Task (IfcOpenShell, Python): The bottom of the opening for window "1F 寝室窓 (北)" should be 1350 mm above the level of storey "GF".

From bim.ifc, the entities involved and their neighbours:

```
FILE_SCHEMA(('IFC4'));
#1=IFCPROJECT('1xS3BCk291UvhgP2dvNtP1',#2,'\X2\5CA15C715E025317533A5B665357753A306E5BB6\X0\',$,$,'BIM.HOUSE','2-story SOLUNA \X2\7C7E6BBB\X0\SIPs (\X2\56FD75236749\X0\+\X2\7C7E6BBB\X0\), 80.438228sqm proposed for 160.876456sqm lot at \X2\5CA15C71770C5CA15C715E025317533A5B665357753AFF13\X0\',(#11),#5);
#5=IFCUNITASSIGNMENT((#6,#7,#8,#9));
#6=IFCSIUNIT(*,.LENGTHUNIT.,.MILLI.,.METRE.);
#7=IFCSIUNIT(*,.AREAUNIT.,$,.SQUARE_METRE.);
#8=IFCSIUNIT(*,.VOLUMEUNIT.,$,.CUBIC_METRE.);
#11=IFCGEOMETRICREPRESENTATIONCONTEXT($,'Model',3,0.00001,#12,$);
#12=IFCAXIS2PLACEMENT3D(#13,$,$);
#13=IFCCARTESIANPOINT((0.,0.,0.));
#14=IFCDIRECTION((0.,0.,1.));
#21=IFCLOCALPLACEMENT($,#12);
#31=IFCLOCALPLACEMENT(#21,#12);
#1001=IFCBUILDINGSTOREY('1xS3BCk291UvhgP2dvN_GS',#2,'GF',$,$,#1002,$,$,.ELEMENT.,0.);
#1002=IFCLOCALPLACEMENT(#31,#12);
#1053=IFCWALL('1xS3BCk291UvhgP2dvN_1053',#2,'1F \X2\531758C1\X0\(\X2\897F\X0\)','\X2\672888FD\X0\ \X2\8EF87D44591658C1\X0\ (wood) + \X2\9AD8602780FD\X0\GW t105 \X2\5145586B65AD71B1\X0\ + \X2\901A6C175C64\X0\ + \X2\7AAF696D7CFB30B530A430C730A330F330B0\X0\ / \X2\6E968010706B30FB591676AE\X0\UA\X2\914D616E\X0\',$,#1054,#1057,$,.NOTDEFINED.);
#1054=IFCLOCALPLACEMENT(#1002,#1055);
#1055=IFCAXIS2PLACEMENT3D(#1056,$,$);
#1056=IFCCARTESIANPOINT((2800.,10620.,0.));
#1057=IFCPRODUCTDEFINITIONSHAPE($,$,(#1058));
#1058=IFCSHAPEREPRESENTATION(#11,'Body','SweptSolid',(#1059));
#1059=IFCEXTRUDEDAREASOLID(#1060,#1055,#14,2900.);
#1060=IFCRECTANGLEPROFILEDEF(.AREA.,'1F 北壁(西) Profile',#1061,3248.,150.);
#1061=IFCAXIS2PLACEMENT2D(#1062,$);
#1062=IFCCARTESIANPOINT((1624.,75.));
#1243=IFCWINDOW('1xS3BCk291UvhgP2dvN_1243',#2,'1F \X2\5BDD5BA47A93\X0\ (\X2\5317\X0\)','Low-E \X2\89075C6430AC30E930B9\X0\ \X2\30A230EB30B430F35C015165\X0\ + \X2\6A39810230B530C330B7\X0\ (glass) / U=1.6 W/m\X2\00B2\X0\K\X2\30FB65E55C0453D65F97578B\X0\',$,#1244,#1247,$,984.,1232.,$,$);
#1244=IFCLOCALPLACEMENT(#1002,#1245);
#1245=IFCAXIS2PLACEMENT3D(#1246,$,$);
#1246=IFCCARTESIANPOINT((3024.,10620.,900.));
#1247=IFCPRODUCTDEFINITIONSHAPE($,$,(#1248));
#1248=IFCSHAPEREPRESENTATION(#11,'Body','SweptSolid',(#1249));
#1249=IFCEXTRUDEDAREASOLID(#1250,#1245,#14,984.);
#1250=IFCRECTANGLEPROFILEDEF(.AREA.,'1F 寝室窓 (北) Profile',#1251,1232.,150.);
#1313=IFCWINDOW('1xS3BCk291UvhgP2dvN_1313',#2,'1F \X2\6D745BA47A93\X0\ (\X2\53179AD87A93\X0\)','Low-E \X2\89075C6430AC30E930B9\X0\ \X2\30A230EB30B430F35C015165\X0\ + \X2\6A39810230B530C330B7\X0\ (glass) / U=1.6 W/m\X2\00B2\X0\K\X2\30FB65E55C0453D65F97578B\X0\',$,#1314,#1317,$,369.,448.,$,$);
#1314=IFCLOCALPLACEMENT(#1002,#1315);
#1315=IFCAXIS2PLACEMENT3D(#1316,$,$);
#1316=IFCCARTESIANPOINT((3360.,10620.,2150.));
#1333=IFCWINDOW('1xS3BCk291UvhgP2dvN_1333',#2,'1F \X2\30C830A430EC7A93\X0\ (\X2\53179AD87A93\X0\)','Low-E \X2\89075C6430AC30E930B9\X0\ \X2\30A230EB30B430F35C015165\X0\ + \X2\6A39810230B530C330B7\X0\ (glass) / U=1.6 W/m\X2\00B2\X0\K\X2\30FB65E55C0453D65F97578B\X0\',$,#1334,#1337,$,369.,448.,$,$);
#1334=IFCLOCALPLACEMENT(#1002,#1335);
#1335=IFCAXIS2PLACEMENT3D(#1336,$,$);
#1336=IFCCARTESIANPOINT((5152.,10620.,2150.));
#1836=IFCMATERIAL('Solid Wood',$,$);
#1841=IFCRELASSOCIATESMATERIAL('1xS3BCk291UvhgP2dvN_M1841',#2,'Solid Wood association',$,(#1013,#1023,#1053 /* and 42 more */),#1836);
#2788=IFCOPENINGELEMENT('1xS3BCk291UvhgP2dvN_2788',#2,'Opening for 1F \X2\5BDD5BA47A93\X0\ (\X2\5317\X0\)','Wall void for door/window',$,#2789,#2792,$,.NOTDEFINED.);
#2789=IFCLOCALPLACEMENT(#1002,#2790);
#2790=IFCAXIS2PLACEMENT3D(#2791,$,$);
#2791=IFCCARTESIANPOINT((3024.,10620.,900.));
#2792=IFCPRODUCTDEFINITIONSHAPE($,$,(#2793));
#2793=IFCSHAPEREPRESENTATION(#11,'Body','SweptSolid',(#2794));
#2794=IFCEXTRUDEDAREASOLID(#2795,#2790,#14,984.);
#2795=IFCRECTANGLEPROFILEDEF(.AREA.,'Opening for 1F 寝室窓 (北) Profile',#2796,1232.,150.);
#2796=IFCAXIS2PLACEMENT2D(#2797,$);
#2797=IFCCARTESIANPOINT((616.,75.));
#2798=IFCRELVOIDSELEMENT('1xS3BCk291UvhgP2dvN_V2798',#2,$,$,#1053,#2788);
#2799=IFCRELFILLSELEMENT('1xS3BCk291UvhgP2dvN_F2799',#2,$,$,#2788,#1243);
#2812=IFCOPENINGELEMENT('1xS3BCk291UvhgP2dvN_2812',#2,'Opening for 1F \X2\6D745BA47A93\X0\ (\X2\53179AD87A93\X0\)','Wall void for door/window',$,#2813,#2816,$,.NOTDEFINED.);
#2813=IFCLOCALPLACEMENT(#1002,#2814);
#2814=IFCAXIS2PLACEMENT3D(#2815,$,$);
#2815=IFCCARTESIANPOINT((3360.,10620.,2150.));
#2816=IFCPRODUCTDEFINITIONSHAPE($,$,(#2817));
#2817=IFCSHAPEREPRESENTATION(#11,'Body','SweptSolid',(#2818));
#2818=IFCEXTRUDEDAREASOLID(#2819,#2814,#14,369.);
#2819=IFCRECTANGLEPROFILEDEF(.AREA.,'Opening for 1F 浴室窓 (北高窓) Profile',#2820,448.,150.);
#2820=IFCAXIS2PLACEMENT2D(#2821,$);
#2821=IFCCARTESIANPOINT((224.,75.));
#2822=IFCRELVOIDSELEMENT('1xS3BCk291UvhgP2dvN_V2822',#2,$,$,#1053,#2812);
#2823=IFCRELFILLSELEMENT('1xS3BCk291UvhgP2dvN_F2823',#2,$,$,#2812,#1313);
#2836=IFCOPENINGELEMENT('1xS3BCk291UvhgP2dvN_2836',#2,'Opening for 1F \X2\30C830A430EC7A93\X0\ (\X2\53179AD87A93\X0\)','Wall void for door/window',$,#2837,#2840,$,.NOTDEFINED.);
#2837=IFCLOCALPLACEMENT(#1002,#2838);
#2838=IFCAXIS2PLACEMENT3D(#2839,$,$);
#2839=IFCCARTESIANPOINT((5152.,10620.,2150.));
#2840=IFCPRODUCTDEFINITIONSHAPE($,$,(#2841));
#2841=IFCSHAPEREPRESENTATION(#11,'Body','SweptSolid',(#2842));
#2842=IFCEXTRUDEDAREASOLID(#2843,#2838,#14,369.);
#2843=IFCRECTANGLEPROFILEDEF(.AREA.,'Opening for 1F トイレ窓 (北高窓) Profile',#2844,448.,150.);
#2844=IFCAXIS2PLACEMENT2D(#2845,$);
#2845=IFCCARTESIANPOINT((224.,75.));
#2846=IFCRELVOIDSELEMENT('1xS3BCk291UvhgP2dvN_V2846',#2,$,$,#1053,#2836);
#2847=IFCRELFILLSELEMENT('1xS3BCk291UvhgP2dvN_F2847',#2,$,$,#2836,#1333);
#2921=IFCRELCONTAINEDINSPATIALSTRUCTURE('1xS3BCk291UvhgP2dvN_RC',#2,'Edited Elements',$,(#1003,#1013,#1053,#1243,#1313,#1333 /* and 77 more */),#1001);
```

```python
import numpy as np
import ifcopenshell
import ifcopenshell.api.geometry
import ifcopenshell.geom
import ifcopenshell.util.element
import ifcopenshell.util.placement
import ifcopenshell.util.shape
import ifcopenshell.util.unit

model = ifcopenshell.open("bim.ifc")
unit_scale = ifcopenshell.util.unit.calculate_unit_scale(model)

window = model.by_guid("1xS3BCk291UvhgP2dvN_1243")
opening = window.FillsVoids[0].RelatingOpeningElement
storey = ifcopenshell.util.element.get_container(window, ifc_class="IfcBuildingStorey")
level = ifcopenshell.util.placement.get_local_placement(storey.ObjectPlacement)[2, 3]

# The opening's origin need not be at the sill, so measure its lowest point.
shape = ifcopenshell.geom.create_shape(ifcopenshell.geom.settings(), opening)
bottom = ifcopenshell.util.shape.get_shape_bottom_elevation(shape, shape.geometry) / unit_scale
dz = level + 1.35 / unit_scale - bottom

shift = np.array([0.0, 0.0, dz])
# The window is not placed relative to its opening, so move both.
for product in (opening, window):
    matrix = ifcopenshell.util.placement.get_local_placement(product.ObjectPlacement)
    matrix[:3, 3] += shift
    ifcopenshell.api.geometry.edit_object_placement(model, product=product, matrix=matrix, is_si=False)

print(f"moved by {dz * unit_scale:+.3f} m")

model.write("bim_updated.ifc")
```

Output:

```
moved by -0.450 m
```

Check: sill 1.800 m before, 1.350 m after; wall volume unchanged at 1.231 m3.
